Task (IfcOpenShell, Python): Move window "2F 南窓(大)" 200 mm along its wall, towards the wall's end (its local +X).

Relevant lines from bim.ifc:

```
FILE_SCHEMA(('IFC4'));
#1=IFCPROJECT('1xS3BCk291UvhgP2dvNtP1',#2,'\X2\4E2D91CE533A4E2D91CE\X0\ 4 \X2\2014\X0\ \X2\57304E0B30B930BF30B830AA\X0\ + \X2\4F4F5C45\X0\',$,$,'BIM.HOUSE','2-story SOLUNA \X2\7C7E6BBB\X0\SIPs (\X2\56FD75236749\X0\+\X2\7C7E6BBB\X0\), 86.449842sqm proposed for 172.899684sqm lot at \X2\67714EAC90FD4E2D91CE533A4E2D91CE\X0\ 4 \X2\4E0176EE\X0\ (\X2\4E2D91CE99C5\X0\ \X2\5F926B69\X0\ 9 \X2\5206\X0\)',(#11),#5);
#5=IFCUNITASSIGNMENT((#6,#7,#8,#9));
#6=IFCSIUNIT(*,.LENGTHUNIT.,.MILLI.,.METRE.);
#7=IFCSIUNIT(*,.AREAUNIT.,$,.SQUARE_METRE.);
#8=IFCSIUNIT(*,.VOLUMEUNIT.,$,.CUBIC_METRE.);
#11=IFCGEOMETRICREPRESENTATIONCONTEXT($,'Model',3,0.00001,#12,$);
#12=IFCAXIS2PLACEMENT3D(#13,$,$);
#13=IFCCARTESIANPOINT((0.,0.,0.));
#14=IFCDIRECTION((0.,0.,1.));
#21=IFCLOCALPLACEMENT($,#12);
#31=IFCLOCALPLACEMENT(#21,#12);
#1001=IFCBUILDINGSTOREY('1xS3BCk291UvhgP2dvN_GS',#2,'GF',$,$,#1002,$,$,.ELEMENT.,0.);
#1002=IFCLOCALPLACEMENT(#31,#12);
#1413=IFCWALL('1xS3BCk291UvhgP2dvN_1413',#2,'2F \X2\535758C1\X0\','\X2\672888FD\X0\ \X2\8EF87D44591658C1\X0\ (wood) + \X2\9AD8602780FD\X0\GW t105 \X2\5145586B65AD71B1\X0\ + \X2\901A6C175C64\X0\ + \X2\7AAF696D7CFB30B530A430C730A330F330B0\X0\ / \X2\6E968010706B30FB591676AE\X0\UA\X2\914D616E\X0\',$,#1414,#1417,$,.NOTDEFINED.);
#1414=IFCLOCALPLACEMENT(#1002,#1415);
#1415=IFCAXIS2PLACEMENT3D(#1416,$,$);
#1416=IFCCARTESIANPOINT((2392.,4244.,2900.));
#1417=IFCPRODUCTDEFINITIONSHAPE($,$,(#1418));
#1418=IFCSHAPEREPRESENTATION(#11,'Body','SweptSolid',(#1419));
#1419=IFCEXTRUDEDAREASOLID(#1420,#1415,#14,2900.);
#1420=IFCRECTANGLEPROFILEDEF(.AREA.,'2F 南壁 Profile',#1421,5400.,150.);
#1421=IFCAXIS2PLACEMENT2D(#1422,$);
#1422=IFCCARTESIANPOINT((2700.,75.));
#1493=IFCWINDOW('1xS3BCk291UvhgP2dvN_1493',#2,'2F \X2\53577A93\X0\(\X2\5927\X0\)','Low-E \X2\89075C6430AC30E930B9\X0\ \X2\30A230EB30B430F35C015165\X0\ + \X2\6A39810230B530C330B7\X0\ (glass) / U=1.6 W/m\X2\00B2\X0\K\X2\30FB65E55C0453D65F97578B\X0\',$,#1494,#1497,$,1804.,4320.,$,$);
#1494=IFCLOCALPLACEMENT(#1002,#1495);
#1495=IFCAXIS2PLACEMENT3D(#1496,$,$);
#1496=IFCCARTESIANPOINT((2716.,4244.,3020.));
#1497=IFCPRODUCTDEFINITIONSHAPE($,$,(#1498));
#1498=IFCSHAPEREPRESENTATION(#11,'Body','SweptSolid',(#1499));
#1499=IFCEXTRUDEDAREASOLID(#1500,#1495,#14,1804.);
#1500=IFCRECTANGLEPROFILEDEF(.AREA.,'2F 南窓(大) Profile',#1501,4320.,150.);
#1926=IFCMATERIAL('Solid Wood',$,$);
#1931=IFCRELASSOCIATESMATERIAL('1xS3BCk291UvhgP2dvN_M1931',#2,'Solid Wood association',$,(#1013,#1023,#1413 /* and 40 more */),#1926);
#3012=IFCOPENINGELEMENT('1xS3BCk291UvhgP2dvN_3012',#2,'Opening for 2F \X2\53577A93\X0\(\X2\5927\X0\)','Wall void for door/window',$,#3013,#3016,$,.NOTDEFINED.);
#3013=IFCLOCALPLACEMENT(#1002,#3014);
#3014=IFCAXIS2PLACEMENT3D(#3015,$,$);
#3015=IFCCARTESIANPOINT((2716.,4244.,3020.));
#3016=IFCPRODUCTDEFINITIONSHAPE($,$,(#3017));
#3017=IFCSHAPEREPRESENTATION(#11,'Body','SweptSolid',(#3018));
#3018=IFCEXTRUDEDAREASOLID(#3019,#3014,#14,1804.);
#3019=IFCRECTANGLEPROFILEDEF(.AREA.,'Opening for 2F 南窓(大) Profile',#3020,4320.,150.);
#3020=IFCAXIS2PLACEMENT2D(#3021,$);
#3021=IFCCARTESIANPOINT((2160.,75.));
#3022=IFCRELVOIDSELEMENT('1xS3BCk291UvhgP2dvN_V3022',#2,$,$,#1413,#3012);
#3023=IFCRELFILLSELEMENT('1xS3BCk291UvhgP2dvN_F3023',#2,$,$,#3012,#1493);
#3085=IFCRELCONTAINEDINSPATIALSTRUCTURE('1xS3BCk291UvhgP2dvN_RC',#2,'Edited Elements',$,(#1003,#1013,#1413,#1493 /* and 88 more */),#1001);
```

```python
import ifcopenshell
import ifcopenshell.api.geometry
import ifcopenshell.util.placement
import ifcopenshell.util.unit

model = ifcopenshell.open("bim.ifc")
unit_scale = ifcopenshell.util.unit.calculate_unit_scale(model)

window = model.by_guid("1xS3BCk291UvhgP2dvN_1493")
opening = window.FillsVoids[0].RelatingOpeningElement
wall = opening.VoidsElements[0].RelatingBuildingElement

wall_matrix = ifcopenshell.util.placement.get_local_placement(wall.ObjectPlacement)
shift = wall_matrix[:3, 0] * 0.2 / unit_scale
before = ifcopenshell.util.placement.get_local_placement(window.ObjectPlacement)[:3, 3].copy()

# The window is not placed relative to its opening, so move both.
for product in (opening, window):
    matrix = ifcopenshell.util.placement.get_local_placement(product.ObjectPlacement)
    matrix[:3, 3] += shift
    ifcopenshell.api.geometry.edit_object_placement(model, product=product, matrix=matrix, is_si=False)

after = ifcopenshell.util.placement.get_local_placement(window.ObjectPlacement)[:3, 3]
print("window moved by", (after - before).round(3) + 0.0)

model.write("bim-out.ifc")
```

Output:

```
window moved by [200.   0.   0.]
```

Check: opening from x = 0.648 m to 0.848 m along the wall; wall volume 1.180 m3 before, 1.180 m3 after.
